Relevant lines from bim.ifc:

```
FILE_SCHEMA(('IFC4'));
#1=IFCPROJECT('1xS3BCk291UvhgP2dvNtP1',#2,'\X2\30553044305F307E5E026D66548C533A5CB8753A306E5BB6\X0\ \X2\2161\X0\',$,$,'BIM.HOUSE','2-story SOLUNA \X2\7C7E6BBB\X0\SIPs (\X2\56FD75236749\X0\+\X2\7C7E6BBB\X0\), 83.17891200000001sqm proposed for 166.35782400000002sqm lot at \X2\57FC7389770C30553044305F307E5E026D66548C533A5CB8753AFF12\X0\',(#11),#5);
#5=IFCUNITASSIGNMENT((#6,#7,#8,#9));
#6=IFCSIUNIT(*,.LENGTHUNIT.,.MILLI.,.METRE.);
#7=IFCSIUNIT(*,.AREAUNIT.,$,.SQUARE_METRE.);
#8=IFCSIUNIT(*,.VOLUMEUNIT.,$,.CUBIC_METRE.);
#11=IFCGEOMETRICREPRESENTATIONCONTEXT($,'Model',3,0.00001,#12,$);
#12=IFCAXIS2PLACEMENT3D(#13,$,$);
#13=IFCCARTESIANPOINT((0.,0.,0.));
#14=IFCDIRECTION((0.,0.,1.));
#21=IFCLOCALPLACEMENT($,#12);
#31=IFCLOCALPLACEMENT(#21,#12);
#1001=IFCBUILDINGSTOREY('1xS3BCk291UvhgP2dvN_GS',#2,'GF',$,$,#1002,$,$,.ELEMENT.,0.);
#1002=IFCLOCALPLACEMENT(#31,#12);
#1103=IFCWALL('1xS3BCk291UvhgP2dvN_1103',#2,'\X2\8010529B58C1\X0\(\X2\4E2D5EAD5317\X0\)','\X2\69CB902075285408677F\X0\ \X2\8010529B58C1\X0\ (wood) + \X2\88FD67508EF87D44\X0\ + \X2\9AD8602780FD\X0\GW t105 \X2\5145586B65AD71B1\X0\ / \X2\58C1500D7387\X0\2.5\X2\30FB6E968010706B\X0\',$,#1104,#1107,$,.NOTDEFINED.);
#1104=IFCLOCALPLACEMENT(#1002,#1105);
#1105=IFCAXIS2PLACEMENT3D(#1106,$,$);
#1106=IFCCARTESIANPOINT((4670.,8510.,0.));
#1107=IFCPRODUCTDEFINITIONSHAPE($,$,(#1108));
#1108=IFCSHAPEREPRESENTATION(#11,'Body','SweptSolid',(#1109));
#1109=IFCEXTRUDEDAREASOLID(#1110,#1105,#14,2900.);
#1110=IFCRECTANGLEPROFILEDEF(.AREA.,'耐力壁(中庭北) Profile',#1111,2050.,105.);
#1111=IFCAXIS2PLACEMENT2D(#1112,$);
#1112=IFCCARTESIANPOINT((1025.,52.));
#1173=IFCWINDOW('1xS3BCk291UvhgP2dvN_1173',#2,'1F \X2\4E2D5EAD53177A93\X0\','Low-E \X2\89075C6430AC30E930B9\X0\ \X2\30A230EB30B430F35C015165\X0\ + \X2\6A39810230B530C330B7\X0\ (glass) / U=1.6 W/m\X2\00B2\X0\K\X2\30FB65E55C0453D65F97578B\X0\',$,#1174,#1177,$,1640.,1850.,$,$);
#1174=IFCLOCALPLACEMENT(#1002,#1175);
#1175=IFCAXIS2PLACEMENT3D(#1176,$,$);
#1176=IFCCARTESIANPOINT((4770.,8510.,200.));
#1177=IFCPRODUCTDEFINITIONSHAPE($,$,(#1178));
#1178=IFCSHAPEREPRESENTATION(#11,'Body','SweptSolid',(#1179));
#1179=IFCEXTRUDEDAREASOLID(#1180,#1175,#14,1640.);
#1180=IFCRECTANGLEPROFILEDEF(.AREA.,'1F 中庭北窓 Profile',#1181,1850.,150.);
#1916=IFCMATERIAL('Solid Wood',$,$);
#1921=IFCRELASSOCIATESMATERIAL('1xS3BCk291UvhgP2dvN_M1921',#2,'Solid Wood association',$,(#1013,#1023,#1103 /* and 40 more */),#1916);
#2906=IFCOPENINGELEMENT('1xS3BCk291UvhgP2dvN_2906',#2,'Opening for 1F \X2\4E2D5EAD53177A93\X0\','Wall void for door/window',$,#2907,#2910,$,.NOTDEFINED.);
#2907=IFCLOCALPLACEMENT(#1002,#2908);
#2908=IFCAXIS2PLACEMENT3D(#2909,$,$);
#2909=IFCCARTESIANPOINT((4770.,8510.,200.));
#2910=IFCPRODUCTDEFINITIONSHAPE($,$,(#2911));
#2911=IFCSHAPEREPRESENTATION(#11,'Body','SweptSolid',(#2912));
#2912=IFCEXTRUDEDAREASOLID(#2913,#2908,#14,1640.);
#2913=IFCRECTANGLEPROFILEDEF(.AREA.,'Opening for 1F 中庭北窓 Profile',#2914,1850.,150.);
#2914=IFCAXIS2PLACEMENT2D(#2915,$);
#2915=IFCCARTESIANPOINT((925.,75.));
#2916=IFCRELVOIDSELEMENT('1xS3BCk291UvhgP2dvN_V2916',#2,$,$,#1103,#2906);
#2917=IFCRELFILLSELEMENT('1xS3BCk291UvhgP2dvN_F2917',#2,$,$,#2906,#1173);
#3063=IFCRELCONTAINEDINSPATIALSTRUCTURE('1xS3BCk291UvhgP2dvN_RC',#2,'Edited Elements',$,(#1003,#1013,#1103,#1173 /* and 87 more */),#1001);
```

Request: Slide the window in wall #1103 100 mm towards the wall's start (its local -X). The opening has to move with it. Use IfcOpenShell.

```python
import ifcopenshell
import ifcopenshell.api.geometry
import ifcopenshell.util.placement

model = ifcopenshell.open("bim.ifc")

window = model.by_guid("1xS3BCk291UvhgP2dvN_1173")
opening = window.FillsVoids[0].RelatingOpeningElement
wall = opening.VoidsElements[0].RelatingBuildingElement

wall_matrix = ifcopenshell.util.placement.get_local_placement(wall.ObjectPlacement)
shift = wall_matrix[:3, 0] * -100.0
before = ifcopenshell.util.placement.get_local_placement(window.ObjectPlacement)[:3, 3].copy()

# The window is not placed relative to its opening, so move both.
for product in (opening, window):
    matrix = ifcopenshell.util.placement.get_local_placement(product.ObjectPlacement)
    matrix[:3, 3] += shift
    ifcopenshell.api.geometry.edit_object_placement(model, product=product, matrix=matrix, is_si=False)

after = ifcopenshell.util.placement.get_local_placement(window.ObjectPlacement)[:3, 3]
print("window moved by", (after - before).round(3) + 0.0)

model.write("bim-out.ifc")
```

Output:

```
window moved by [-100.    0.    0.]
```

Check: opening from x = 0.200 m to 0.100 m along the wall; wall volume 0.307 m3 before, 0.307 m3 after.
